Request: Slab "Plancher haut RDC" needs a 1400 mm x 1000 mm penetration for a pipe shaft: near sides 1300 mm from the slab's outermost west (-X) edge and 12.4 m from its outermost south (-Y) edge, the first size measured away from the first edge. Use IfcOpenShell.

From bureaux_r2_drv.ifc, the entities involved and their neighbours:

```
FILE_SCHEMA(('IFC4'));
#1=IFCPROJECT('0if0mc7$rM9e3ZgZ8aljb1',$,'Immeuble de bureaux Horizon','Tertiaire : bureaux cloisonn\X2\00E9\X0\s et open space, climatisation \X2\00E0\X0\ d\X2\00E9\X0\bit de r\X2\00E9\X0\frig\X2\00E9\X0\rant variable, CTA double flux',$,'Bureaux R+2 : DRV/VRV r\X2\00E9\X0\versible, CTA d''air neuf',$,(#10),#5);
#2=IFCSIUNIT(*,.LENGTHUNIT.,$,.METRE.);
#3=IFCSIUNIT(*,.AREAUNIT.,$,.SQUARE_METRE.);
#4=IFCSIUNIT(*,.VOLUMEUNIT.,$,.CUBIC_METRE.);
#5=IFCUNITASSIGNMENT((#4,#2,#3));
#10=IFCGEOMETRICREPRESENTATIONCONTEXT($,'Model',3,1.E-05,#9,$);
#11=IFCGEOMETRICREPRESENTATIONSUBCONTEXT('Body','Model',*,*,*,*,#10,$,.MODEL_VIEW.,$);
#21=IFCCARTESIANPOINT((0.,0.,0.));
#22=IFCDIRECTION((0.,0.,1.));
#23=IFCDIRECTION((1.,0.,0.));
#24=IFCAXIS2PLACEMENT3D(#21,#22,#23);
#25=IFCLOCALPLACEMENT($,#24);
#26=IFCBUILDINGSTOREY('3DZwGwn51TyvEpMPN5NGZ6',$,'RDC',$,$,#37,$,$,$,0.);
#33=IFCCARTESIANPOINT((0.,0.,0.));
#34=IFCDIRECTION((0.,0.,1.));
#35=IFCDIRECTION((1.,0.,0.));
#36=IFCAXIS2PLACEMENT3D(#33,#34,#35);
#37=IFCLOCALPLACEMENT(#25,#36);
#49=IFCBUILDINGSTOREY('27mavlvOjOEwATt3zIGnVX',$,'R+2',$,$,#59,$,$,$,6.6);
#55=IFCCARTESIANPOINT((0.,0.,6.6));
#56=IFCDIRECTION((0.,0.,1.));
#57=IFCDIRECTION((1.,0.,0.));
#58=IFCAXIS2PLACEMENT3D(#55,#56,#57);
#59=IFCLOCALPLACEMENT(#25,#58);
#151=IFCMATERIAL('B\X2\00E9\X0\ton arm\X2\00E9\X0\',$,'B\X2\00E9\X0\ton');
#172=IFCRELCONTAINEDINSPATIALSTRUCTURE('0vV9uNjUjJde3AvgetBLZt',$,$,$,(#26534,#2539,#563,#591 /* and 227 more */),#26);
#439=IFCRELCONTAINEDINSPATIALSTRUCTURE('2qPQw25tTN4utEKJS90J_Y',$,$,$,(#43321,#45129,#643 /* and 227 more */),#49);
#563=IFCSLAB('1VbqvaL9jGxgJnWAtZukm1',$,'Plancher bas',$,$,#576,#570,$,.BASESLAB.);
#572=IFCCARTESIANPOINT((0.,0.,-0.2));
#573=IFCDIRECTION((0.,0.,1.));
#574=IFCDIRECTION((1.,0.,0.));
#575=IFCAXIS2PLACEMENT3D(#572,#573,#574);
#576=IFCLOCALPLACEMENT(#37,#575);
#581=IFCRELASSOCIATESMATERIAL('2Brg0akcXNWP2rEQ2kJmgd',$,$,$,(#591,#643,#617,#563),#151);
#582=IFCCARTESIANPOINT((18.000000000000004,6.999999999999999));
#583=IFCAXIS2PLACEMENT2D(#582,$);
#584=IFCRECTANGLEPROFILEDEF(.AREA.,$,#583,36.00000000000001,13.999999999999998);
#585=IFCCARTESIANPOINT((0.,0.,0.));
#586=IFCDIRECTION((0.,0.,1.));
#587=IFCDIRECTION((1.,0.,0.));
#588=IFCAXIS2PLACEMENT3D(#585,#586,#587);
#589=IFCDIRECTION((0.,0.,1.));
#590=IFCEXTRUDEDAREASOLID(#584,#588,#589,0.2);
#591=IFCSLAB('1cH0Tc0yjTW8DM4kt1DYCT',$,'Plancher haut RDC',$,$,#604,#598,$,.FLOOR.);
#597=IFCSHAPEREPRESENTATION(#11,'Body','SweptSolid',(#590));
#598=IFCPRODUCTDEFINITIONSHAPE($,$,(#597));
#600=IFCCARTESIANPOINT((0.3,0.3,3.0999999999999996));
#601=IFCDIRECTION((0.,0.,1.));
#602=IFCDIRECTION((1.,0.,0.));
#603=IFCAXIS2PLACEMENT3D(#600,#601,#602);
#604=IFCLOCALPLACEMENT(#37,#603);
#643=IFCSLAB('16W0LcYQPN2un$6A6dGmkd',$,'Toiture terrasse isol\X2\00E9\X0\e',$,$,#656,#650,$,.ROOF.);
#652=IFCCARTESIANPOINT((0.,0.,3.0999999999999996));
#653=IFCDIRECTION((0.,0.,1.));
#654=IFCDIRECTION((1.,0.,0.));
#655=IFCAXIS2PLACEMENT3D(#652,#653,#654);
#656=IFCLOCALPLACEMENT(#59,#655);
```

```python
import numpy as np
import ifcopenshell
import ifcopenshell.api.feature
import ifcopenshell.api.geometry
import ifcopenshell.api.root
import ifcopenshell.geom
import ifcopenshell.util.placement
import ifcopenshell.util.representation
import ifcopenshell.util.shape
import ifcopenshell.util.unit

model = ifcopenshell.open("bureaux_r2_drv.ifc")
unit_scale = ifcopenshell.util.unit.calculate_unit_scale(model)
settings = ifcopenshell.geom.settings()


def volume(element):
    """Net volume in cubic metres, openings subtracted."""
    shape = ifcopenshell.geom.create_shape(settings, element)
    return ifcopenshell.util.shape.get_volume(shape.geometry)


slab = model.by_guid("1cH0Tc0yjTW8DM4kt1DYCT")
before = volume(slab)

# Extent in the slab's own axes, in metres. The edges named are its -X and -Y sides.
slab_shape = ifcopenshell.geom.create_shape(settings, slab)
vertices = ifcopenshell.util.shape.get_vertices(slab_shape.geometry)
x_min, y_min, bottom = vertices.min(axis=0)
top = vertices[:, 2].max()

opening = ifcopenshell.api.root.create_entity(model, ifc_class="IfcOpeningElement", name="Pipe shaft opening", predefined_type="OPENING")
context = ifcopenshell.util.representation.get_context(model, "Model", "Body", "MODEL_VIEW")
width, depth = 1.4, 1
outline = [(0.0, 0.0), (width, 0.0), (width, depth), (0.0, depth), (0.0, 0.0)]
# Overshoot both faces by 50 mm so the cut is clean.
shape = ifcopenshell.api.geometry.add_slab_representation(
    model, context=context, depth=top - bottom + 0.1, polyline=outline
)
ifcopenshell.api.geometry.assign_representation(model, product=opening, representation=shape)

matrix = ifcopenshell.util.placement.get_local_placement(slab.ObjectPlacement)
matrix[:, 3] = matrix @ np.append(np.array([x_min + 1.3, y_min + 12.4, bottom - 0.05]) / unit_scale, 1.0)
ifcopenshell.api.geometry.edit_object_placement(model, product=opening, matrix=matrix, is_si=False)
ifcopenshell.api.feature.add_feature(model, feature=opening, element=slab)

after = volume(slab)

print(f"slab volume {before:.3f} -> {after:.3f} m3")

model.write("bureaux_r2_drv-out.ifc")
```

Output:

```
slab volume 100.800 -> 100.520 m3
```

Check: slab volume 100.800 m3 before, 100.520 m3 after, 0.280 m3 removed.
